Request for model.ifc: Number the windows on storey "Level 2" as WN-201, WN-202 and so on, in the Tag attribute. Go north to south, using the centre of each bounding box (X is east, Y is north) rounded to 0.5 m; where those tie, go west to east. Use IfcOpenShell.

First a look at what the model holds.

```python
import ifcopenshell
import ifcopenshell.util.element
import ifcopenshell.util.placement

model = ifcopenshell.open("model.ifc")
print(model.schema)
storey = next(s for s in model.by_type("IfcBuildingStorey") if s.Name == "Level 2")
windows = [e for e in ifcopenshell.util.element.get_decomposition(storey) if e.is_a("IfcWindow")]
for e in sorted(windows, key=lambda e: e.id()):
    origin = ifcopenshell.util.placement.get_local_placement(e.ObjectPlacement)[:3, 3]
    print(e.id(), e.Tag, e.Name, origin.round(2) + 0.0, sep=" | ")
```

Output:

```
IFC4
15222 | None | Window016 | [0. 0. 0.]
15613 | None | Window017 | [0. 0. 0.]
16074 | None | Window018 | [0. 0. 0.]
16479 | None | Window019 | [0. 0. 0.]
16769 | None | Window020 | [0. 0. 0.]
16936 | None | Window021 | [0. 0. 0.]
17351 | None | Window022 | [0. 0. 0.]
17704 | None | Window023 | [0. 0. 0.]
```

```python
import ifcopenshell
import ifcopenshell.geom
import ifcopenshell.util.element
import ifcopenshell.util.shape

model = ifcopenshell.open("model.ifc")
settings = ifcopenshell.geom.settings()
settings.set("use-world-coords", True)


def centre(element):
    shape = ifcopenshell.geom.create_shape(settings, element)
    return ifcopenshell.util.shape.get_bbox_centroid(shape.geometry)


storey = next(s for s in model.by_type("IfcBuildingStorey") if s.Name == "Level 2")
windows = [e for e in ifcopenshell.util.element.get_decomposition(storey) if e.is_a("IfcWindow")]

# Insertion points can sit at a corner or the storey origin, so sort by the geometry (in metres).
centres = {e: centre(e) for e in windows}
windows.sort(key=lambda e: (-round(centres[e][1] / 0.5), centres[e][0]))

for i, e in enumerate(windows, start=1):
    number = f"WN-2{i:02d}"
    e.Tag = number
    print(e.id(), number)

model.write("model_v2.ifc")
```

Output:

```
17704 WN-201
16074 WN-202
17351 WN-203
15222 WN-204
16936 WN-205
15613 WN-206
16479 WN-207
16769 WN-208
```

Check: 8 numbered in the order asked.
